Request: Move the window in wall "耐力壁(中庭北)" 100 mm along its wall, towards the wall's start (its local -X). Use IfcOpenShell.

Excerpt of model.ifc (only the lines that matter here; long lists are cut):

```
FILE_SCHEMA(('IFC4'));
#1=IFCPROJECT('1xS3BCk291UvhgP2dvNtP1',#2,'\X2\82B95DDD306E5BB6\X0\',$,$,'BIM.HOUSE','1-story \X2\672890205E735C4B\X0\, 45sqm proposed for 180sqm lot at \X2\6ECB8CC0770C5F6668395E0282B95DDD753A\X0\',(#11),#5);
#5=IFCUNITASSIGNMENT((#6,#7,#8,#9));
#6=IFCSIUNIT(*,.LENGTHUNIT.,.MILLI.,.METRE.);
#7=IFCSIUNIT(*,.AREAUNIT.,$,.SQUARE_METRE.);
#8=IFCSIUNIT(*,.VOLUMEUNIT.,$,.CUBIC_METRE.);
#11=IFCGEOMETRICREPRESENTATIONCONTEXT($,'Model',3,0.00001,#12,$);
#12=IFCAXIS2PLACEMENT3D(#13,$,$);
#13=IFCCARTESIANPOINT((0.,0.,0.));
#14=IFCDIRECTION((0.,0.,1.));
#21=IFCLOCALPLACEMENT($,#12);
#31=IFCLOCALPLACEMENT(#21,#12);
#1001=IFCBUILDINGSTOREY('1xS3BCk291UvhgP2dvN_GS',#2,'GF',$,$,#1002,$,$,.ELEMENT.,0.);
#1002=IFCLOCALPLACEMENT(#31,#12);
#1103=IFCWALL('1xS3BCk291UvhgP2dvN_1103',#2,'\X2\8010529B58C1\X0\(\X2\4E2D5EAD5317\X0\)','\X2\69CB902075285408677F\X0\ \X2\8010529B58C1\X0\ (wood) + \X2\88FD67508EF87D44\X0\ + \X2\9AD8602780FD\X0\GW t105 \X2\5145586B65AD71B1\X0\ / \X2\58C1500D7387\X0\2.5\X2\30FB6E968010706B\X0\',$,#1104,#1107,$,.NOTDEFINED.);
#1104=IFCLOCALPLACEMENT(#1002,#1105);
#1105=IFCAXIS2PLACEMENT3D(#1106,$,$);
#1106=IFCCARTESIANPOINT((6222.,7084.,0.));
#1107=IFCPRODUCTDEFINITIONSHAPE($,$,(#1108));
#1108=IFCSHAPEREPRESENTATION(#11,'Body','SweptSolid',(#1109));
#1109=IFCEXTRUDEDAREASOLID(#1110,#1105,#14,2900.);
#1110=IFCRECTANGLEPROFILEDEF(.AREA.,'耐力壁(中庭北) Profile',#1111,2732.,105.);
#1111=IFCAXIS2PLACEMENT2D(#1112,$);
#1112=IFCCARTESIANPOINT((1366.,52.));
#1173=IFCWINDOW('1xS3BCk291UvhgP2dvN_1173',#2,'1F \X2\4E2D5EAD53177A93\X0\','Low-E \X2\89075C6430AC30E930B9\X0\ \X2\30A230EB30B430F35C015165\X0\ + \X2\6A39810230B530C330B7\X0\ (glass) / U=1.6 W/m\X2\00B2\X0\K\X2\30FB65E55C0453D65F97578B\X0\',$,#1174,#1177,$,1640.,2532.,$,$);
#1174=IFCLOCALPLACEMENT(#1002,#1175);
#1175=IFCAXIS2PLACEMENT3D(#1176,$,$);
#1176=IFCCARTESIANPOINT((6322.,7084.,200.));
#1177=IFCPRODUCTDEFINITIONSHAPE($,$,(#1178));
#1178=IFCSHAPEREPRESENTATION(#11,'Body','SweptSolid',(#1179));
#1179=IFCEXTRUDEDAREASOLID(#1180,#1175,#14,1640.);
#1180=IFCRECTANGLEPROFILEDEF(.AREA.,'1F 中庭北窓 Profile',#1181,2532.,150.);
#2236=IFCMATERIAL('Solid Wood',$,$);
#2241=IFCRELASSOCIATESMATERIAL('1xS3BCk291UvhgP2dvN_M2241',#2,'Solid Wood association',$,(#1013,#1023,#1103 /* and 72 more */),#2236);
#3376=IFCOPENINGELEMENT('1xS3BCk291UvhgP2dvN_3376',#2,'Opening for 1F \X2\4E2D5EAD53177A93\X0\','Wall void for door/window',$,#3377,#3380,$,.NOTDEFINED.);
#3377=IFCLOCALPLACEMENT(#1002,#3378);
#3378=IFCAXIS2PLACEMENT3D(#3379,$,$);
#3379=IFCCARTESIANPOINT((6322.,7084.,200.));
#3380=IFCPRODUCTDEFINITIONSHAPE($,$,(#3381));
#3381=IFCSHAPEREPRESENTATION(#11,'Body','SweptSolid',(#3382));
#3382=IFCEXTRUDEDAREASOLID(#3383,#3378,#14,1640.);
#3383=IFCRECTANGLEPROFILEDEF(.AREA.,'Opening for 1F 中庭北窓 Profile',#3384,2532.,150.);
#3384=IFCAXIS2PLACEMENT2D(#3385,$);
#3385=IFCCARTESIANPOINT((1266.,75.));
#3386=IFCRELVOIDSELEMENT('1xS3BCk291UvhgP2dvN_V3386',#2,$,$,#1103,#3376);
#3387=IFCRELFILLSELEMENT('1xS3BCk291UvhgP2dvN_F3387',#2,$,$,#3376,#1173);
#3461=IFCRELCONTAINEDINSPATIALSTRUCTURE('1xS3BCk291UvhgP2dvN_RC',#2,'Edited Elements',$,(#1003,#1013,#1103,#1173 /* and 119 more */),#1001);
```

```python
import ifcopenshell
import ifcopenshell.api.geometry
import ifcopenshell.util.placement

model = ifcopenshell.open("model.ifc")

window = model.by_guid("1xS3BCk291UvhgP2dvN_1173")
opening = window.FillsVoids[0].RelatingOpeningElement
wall = opening.VoidsElements[0].RelatingBuildingElement

wall_matrix = ifcopenshell.util.placement.get_local_placement(wall.ObjectPlacement)
shift = wall_matrix[:3, 0] * -100.0
before = ifcopenshell.util.placement.get_local_placement(window.ObjectPlacement)[:3, 3].copy()

# The window is not placed relative to its opening, so move both.
for product in (opening, window):
    matrix = ifcopenshell.util.placement.get_local_placement(product.ObjectPlacement)
    matrix[:3, 3] += shift
    ifcopenshell.api.geometry.edit_object_placement(model, product=product, matrix=matrix, is_si=False)

after = ifcopenshell.util.placement.get_local_placement(window.ObjectPlacement)[:3, 3]
print("window moved by", (after - before).round(3) + 0.0)

model.write("model_v2.ifc")
```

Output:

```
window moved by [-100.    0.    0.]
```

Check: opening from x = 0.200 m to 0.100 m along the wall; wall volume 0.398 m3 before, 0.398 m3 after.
